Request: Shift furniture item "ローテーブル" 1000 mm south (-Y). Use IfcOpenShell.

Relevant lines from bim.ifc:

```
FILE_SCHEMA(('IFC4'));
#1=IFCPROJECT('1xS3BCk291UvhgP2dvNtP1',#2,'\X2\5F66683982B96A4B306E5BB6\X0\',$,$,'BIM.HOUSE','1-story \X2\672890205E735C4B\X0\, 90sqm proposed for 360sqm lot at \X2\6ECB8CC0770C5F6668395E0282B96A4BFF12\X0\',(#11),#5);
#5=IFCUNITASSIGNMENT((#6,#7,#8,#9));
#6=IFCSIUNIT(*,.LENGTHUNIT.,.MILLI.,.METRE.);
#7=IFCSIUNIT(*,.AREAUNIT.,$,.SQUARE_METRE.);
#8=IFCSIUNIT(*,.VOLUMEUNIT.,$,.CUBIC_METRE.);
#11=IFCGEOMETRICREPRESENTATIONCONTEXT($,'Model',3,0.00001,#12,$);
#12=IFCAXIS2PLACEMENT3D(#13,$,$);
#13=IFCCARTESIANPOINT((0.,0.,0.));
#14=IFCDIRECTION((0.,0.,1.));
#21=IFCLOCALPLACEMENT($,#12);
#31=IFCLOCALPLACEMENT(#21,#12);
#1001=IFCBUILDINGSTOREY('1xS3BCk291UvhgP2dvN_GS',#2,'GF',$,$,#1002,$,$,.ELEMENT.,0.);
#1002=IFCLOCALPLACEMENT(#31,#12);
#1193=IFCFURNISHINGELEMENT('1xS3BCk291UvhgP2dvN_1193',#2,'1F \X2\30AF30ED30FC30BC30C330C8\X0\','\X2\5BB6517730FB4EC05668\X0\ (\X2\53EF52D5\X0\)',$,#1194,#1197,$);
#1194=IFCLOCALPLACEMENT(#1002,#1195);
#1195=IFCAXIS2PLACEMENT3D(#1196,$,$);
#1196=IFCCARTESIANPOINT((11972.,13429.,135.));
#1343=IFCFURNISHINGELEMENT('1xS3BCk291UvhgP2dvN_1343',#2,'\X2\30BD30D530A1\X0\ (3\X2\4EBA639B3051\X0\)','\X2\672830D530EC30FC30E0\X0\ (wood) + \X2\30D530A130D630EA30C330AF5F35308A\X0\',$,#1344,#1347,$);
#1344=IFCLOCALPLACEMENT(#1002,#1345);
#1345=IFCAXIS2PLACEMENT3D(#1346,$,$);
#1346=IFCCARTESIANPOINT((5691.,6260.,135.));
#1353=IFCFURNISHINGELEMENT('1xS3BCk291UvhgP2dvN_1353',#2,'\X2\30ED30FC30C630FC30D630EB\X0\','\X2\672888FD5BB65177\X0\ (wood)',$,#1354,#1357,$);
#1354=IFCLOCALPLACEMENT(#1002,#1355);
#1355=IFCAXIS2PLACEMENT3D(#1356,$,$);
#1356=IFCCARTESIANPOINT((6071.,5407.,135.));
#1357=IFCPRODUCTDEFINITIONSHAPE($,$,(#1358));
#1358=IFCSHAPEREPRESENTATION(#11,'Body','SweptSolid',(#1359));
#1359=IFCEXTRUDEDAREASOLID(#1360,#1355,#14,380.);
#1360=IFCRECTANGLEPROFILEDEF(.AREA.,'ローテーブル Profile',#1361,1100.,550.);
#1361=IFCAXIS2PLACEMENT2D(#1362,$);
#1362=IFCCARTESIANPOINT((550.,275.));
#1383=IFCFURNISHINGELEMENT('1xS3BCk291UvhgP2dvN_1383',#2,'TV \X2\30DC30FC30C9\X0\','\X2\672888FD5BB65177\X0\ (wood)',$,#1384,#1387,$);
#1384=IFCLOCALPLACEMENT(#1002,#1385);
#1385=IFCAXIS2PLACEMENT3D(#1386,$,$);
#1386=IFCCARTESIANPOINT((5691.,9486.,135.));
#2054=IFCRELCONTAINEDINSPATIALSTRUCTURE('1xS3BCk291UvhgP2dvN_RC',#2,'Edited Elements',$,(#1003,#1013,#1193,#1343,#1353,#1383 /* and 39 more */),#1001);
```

```python
import ifcopenshell
import ifcopenshell.api.geometry
import ifcopenshell.util.placement

model = ifcopenshell.open("bim.ifc")

item = model.by_guid("1xS3BCk291UvhgP2dvN_1353")
matrix = ifcopenshell.util.placement.get_local_placement(item.ObjectPlacement)
matrix[1, 3] -= 1000.0
ifcopenshell.api.geometry.edit_object_placement(model, product=item, matrix=matrix, is_si=False)

print(ifcopenshell.util.placement.get_local_placement(item.ObjectPlacement).round(3) + 0.0)

model.write("bim_rev.ifc")
```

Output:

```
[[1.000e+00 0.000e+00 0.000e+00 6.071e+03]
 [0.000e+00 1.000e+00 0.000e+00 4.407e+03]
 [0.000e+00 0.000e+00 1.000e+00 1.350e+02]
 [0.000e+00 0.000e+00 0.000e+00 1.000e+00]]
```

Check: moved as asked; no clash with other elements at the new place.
